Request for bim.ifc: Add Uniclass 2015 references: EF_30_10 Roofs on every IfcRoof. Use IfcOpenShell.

First a look at what the model holds.

```python
import ifcopenshell

model = ifcopenshell.open("bim.ifc")
print(model.schema)
print("classifications:", [c.Name for c in model.by_type("IfcClassification")])
for ifc_class in ("IfcDoor", "IfcRoof", "IfcStair", "IfcWall", "IfcWindow"):
    print(ifc_class, len(model.by_type(ifc_class)))
```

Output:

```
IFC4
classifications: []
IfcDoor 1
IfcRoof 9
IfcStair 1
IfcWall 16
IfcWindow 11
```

```python
import ifcopenshell
import ifcopenshell.api.classification

model = ifcopenshell.open("bim.ifc")

system = ifcopenshell.api.classification.add_classification(model, classification="Uniclass 2015")

codes = {
    "IfcRoof": ("EF_30_10", "Roofs"),
}
for ifc_class, (code, name) in codes.items():
    products = model.by_type(ifc_class)
    ifcopenshell.api.classification.add_reference(
        model, products=products, classification=system, identification=code, name=name
    )
    print(code, len(products))

model.write("bim_updated.ifc")
```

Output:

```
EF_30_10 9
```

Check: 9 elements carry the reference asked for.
